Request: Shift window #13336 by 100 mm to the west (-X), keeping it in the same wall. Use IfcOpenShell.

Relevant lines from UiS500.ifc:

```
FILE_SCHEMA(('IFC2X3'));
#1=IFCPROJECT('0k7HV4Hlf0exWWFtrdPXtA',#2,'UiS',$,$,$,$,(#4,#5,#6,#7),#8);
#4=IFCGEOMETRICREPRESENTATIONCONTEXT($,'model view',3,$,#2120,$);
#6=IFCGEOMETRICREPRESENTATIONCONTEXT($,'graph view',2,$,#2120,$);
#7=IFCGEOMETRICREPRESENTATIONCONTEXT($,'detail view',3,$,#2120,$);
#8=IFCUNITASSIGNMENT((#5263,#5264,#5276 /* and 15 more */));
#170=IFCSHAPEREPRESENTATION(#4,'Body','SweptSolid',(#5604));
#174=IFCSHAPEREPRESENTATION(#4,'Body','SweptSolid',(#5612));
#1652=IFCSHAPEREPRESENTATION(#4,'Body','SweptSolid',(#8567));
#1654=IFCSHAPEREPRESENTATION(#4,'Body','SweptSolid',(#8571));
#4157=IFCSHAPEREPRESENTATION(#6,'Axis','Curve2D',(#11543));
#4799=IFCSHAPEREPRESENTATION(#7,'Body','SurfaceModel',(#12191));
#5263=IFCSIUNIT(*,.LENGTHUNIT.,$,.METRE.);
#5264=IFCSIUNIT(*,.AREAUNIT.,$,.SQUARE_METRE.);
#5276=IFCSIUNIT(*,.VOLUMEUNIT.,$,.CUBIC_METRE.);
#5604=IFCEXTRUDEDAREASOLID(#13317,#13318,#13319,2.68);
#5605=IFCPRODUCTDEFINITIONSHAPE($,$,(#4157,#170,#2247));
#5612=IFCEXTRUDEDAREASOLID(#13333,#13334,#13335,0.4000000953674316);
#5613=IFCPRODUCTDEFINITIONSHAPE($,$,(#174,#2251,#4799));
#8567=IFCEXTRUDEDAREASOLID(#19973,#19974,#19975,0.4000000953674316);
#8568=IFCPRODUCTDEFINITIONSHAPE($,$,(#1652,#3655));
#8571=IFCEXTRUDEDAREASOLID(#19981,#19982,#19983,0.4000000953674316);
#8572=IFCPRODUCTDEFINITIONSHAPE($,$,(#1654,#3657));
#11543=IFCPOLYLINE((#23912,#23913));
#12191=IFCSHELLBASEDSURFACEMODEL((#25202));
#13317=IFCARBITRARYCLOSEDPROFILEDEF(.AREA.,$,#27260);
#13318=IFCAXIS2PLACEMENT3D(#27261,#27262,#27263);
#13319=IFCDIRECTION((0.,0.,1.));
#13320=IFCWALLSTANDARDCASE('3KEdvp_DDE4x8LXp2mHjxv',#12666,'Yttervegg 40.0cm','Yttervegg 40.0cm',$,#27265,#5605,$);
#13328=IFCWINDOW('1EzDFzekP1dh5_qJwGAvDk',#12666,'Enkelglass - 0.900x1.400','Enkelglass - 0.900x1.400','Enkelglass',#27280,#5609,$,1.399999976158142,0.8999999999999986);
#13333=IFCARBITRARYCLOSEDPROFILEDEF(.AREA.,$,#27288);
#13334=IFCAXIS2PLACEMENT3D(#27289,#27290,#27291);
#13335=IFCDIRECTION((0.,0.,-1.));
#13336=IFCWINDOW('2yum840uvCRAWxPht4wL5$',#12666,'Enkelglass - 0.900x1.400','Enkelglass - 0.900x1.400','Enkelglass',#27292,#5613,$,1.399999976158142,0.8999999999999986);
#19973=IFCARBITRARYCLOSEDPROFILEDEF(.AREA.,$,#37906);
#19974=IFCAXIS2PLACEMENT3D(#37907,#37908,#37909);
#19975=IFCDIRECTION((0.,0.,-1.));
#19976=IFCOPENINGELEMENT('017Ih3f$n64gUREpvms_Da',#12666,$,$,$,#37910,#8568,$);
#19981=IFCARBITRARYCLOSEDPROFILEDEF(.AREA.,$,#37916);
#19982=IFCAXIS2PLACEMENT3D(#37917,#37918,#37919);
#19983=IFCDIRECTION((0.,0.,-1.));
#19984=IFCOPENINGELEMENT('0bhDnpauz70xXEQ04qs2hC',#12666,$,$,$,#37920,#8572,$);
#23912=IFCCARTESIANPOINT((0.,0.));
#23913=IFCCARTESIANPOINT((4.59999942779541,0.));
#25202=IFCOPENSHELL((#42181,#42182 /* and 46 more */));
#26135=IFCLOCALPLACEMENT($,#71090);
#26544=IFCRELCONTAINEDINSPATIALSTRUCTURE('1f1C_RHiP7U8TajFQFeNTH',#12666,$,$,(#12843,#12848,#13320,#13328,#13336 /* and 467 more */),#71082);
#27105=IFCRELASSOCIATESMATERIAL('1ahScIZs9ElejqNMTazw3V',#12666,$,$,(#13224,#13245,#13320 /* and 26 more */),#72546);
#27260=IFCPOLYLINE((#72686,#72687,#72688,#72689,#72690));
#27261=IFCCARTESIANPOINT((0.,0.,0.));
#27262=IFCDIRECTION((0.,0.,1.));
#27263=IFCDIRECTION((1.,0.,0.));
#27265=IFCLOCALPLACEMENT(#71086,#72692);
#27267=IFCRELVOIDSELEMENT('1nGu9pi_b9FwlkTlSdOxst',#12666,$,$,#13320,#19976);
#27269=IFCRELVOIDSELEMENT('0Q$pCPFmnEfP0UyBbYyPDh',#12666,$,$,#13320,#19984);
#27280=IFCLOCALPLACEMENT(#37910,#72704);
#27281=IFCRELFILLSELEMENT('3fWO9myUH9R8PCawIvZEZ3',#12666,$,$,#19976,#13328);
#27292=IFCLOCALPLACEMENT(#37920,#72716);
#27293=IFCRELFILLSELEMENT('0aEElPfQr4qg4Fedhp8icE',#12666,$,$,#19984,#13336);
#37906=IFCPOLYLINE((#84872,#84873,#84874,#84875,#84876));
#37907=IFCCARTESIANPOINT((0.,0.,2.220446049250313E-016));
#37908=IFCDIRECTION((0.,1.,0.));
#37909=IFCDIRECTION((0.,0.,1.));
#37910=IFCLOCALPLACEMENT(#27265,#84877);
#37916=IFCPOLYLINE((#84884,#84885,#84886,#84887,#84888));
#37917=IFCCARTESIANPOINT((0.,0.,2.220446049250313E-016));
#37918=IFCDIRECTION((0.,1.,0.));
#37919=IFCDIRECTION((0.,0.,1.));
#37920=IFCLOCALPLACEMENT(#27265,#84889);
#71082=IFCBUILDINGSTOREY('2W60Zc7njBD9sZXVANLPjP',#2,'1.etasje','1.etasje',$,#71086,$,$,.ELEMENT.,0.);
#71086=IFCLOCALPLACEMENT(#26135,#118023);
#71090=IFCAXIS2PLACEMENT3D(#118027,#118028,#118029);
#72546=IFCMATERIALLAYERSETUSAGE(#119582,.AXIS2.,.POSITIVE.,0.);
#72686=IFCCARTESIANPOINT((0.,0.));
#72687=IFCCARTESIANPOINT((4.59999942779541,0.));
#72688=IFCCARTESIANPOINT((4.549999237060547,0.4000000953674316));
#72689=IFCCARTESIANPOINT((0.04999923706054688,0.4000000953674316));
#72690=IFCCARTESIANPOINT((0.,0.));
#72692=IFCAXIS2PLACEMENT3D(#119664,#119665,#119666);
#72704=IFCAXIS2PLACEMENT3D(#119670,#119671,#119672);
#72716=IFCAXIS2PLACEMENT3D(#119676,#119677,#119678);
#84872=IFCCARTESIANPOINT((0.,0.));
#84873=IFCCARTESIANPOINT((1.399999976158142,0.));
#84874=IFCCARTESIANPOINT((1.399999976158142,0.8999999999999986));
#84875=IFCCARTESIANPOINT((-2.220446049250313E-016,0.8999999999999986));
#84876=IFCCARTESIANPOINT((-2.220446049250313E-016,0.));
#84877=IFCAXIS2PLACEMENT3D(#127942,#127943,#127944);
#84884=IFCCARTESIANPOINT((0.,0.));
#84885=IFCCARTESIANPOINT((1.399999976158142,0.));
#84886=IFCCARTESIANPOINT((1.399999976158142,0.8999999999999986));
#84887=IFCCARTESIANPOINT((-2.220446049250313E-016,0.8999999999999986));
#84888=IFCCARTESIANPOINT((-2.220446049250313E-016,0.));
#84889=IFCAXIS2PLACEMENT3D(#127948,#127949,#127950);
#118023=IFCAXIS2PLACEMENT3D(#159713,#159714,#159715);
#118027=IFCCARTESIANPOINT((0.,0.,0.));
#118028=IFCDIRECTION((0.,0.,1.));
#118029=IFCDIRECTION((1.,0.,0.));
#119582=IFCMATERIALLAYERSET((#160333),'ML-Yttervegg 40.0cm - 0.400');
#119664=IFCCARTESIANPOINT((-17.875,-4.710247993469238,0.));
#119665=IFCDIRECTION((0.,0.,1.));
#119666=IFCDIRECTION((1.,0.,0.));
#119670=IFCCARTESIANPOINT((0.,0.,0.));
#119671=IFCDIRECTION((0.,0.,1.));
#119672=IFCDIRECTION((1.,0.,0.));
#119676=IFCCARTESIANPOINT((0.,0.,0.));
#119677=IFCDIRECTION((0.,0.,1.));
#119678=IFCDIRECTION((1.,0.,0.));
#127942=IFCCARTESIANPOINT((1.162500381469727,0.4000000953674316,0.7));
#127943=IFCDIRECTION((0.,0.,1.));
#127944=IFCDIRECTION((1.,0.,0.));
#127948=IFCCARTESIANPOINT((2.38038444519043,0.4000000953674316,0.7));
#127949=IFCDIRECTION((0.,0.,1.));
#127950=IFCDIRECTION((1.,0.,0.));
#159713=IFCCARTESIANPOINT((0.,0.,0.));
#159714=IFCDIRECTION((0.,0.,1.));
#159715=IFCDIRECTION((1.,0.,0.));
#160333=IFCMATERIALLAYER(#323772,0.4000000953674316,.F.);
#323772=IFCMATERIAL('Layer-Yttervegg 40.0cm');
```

```python
import ifcopenshell
import ifcopenshell.api.geometry
import ifcopenshell.util.placement

model = ifcopenshell.open("UiS500.ifc")

window = model.by_id(13336)
opening = window.FillsVoids[0].RelatingOpeningElement
wall = opening.VoidsElements[0].RelatingBuildingElement

wall_matrix = ifcopenshell.util.placement.get_local_placement(wall.ObjectPlacement)
shift = wall_matrix[:3, 0] * -0.1
before = ifcopenshell.util.placement.get_local_placement(window.ObjectPlacement)[:3, 3].copy()

# The window is placed relative to its opening, so it follows when the opening moves.
matrix = ifcopenshell.util.placement.get_local_placement(opening.ObjectPlacement)
matrix[:3, 3] += shift
ifcopenshell.api.geometry.edit_object_placement(
    model, product=opening, matrix=matrix, is_si=False, should_transform_children=True
)

after = ifcopenshell.util.placement.get_local_placement(window.ObjectPlacement)[:3, 3]
print("window moved by", (after - before).round(3) + 0.0)

model.write("UiS500_v2.ifc")
```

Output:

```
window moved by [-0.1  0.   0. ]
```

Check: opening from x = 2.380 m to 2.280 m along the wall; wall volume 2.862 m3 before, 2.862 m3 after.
